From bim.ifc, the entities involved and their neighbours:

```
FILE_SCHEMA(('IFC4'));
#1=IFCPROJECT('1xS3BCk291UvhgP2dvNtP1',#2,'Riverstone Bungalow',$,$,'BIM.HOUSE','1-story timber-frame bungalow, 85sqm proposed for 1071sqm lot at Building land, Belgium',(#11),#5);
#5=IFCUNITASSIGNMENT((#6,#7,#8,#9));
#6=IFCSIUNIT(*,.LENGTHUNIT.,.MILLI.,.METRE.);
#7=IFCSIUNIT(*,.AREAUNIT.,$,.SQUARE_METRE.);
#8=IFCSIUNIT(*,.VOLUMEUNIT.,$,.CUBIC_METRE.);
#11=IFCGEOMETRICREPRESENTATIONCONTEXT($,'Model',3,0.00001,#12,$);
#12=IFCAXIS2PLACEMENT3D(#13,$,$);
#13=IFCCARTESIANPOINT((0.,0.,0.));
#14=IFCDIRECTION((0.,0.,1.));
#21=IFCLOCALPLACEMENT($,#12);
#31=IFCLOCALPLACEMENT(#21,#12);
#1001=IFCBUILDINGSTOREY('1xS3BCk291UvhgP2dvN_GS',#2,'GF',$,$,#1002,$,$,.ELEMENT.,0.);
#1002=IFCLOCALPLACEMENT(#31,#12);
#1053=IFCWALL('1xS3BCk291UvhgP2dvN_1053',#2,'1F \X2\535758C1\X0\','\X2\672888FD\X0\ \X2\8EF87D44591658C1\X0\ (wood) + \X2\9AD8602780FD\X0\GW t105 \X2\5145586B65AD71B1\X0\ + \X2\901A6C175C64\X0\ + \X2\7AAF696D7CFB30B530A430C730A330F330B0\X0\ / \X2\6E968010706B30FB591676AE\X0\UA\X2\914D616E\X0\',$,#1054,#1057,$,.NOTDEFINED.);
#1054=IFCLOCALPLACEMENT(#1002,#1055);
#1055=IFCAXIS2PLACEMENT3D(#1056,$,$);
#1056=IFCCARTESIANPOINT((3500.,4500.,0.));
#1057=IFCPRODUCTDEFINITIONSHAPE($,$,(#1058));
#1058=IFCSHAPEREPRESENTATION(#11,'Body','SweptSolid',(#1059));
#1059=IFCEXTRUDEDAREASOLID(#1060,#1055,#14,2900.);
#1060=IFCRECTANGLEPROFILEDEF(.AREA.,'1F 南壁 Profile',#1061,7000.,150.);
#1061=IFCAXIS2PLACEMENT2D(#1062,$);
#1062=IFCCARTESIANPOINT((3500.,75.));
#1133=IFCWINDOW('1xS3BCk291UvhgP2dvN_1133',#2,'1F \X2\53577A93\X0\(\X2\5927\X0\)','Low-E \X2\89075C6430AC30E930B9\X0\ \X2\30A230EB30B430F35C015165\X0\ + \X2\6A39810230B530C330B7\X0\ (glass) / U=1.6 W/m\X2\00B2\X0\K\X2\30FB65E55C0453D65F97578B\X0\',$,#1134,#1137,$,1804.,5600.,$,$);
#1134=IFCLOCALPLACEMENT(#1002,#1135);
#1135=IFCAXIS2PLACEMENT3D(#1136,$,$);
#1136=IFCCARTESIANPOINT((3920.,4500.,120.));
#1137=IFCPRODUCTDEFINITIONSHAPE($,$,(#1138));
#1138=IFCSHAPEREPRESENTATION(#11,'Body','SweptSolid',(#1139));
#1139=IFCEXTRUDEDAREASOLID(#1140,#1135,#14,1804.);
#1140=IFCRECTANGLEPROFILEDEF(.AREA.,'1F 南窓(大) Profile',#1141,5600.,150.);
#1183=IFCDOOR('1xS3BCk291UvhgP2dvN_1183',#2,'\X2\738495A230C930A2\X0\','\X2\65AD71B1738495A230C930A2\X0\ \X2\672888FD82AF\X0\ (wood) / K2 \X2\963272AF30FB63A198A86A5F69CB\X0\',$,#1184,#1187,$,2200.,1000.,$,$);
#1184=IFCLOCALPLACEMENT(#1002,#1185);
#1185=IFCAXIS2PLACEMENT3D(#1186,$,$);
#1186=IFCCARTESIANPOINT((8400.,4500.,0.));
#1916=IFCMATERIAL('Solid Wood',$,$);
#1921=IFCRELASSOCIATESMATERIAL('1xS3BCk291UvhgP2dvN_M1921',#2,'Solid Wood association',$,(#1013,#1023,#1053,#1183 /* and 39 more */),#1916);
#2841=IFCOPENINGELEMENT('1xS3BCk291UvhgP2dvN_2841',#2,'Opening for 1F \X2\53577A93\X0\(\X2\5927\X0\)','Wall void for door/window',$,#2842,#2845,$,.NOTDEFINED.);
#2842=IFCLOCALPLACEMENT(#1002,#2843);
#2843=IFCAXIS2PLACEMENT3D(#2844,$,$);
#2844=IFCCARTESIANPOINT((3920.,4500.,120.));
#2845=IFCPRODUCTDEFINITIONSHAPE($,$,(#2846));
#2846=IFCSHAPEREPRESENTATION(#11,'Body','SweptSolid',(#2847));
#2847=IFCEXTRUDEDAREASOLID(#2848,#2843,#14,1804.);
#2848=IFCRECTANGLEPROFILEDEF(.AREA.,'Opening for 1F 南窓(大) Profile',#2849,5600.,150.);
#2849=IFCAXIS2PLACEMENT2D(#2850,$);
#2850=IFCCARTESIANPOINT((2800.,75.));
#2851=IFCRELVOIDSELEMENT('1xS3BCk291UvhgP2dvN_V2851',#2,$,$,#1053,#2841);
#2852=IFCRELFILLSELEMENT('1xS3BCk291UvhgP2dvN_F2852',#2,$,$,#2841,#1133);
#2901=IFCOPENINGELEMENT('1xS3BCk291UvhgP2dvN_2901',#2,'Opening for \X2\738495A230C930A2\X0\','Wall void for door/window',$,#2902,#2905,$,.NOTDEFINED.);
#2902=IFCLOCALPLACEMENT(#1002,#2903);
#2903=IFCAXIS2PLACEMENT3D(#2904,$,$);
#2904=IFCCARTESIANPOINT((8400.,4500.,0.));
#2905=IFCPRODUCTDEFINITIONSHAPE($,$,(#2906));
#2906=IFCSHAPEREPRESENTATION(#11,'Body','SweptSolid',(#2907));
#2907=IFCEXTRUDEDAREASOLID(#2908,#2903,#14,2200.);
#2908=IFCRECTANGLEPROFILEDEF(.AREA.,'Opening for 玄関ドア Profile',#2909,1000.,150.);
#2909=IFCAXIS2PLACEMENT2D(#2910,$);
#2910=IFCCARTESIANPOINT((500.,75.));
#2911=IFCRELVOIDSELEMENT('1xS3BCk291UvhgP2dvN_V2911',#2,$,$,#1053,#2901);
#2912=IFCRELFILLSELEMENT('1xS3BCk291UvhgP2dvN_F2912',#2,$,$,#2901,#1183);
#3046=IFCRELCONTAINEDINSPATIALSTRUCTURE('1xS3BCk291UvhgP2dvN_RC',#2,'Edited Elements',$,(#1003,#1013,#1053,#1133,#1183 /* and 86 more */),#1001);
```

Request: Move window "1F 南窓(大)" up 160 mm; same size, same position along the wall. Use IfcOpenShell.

```python
import numpy as np
import ifcopenshell
import ifcopenshell.api.geometry
import ifcopenshell.util.placement
import ifcopenshell.util.unit

model = ifcopenshell.open("bim.ifc")
unit_scale = ifcopenshell.util.unit.calculate_unit_scale(model)

window = model.by_guid("1xS3BCk291UvhgP2dvN_1133")
opening = window.FillsVoids[0].RelatingOpeningElement
dz = 0.16 / unit_scale

shift = np.array([0.0, 0.0, dz])
# The window is not placed relative to its opening, so move both.
for product in (opening, window):
    matrix = ifcopenshell.util.placement.get_local_placement(product.ObjectPlacement)
    matrix[:3, 3] += shift
    ifcopenshell.api.geometry.edit_object_placement(model, product=product, matrix=matrix, is_si=False)

print(f"moved by {dz * unit_scale:+.3f} m")

model.write("bim_updated.ifc")
```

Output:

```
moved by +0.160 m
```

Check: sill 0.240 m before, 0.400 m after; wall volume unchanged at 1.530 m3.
